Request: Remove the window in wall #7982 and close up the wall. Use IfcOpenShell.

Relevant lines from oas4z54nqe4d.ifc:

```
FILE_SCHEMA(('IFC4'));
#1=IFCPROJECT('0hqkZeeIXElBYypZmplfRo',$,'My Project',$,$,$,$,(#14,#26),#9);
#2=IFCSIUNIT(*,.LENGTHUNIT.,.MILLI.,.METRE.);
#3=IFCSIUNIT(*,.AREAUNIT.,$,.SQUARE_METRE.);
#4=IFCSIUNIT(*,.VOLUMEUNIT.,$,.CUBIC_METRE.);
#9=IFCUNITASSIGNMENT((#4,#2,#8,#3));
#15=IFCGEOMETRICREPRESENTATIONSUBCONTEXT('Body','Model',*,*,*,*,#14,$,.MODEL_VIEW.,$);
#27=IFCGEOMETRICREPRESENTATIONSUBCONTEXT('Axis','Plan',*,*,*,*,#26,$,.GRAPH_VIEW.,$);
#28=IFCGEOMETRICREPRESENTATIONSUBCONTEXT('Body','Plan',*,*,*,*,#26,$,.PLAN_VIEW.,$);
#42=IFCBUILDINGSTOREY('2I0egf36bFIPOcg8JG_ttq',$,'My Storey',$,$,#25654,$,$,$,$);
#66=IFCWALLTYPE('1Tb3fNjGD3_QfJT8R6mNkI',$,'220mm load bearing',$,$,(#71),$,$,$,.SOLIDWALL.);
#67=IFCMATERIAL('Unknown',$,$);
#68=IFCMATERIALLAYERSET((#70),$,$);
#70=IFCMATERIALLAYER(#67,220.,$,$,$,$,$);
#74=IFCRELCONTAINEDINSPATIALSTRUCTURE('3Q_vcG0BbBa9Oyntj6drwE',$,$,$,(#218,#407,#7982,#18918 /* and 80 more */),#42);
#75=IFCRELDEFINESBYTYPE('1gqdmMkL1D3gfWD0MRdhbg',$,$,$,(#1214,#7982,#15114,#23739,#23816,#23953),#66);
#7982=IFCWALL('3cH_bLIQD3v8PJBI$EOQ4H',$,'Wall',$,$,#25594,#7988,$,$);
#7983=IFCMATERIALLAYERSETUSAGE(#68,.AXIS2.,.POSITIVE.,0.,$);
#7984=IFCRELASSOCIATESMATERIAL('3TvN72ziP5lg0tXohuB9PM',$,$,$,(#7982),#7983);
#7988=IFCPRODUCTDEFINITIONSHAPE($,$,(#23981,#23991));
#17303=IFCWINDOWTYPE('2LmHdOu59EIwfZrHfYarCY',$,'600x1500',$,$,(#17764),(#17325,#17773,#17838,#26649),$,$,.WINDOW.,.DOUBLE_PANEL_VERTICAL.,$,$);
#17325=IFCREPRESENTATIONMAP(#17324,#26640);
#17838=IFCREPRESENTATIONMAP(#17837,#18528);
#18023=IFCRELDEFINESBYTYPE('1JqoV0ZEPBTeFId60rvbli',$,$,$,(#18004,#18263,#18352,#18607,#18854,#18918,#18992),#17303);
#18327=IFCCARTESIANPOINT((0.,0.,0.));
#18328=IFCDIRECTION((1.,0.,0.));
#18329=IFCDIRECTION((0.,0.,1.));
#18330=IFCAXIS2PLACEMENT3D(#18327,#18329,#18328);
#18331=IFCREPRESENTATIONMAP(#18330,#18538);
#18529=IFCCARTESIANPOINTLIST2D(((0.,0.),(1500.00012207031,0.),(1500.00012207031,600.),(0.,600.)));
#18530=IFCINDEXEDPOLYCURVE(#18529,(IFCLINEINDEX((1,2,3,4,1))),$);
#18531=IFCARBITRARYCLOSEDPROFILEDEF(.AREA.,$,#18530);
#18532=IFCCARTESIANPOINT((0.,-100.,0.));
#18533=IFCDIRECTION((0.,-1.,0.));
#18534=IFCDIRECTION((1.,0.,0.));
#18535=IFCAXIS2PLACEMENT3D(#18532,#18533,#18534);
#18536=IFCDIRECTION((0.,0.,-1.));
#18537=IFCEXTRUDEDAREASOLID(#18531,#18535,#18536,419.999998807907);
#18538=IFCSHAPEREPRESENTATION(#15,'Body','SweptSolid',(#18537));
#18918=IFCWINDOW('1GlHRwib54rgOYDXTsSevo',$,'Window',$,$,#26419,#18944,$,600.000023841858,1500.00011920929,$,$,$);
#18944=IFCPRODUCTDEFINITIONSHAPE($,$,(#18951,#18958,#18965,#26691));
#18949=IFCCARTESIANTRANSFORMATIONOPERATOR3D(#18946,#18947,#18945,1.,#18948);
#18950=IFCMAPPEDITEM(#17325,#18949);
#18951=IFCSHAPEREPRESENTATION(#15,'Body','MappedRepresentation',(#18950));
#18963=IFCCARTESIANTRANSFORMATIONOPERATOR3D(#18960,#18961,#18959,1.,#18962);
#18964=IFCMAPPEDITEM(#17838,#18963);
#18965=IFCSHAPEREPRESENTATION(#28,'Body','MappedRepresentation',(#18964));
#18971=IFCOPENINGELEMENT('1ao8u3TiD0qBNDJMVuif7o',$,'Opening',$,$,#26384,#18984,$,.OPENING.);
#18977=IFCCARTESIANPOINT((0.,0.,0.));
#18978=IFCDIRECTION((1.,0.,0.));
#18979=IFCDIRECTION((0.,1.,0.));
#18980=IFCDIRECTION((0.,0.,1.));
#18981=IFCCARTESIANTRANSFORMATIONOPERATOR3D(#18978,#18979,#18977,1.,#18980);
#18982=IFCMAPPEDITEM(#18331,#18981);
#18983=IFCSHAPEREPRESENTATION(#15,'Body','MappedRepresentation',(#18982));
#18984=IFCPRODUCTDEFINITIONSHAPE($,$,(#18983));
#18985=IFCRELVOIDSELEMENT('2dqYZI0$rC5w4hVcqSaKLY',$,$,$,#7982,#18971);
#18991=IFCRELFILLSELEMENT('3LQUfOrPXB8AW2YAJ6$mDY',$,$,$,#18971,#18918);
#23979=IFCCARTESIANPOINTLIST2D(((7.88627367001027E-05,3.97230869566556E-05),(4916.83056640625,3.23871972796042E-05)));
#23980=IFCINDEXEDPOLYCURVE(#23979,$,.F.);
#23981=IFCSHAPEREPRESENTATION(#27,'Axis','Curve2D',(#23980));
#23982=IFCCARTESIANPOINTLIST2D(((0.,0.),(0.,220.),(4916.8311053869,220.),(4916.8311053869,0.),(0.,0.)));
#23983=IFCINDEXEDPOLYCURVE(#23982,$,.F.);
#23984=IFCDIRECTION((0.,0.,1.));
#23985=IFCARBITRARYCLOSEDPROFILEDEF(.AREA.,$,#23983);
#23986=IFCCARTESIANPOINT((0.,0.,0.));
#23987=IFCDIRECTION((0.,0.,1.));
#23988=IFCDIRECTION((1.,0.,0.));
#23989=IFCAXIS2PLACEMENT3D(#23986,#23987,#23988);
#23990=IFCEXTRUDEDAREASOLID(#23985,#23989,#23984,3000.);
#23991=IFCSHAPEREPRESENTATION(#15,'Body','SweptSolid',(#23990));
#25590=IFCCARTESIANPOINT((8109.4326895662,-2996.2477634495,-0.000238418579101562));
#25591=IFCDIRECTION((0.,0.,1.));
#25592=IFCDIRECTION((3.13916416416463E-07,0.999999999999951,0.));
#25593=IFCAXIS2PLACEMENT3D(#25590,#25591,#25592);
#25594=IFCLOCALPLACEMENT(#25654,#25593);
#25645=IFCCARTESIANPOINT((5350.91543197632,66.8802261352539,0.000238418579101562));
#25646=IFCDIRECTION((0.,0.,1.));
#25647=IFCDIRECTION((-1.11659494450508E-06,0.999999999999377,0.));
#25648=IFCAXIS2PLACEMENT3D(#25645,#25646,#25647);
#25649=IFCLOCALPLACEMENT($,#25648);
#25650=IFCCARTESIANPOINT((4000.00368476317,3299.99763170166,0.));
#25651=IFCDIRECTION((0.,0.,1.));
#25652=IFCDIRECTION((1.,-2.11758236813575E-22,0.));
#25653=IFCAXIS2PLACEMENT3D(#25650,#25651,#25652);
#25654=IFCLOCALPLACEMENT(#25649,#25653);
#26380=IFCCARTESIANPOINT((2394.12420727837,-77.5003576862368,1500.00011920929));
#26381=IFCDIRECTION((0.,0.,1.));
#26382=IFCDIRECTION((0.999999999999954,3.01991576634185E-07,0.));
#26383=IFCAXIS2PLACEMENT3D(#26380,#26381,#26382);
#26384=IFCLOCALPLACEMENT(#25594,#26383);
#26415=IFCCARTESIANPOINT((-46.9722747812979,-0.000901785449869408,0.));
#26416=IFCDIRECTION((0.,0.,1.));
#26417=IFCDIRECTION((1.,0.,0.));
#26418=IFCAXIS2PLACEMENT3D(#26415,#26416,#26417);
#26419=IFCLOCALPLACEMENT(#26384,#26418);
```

```python
import ifcopenshell
import ifcopenshell.api.feature
import ifcopenshell.api.root
import ifcopenshell.geom
import ifcopenshell.util.shape

model = ifcopenshell.open("oas4z54nqe4d.ifc")
settings = ifcopenshell.geom.settings()


def volume(element):
    """Net volume in cubic metres, openings subtracted."""
    shape = ifcopenshell.geom.create_shape(settings, element)
    return ifcopenshell.util.shape.get_volume(shape.geometry)


window = model.by_guid("1GlHRwib54rgOYDXTsSevo")
opening = window.FillsVoids[0].RelatingOpeningElement
wall = opening.VoidsElements[0].RelatingBuildingElement
before = volume(wall)

ifcopenshell.api.root.remove_product(model, product=window)
ifcopenshell.api.feature.remove_feature(model, feature=opening)

after = volume(wall)

print(f"wall volume {before:.3f} -> {after:.3f} m3")

model.write("oas4z54nqe4d_edited.ifc")
```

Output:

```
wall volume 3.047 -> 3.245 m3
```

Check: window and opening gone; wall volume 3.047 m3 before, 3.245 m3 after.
